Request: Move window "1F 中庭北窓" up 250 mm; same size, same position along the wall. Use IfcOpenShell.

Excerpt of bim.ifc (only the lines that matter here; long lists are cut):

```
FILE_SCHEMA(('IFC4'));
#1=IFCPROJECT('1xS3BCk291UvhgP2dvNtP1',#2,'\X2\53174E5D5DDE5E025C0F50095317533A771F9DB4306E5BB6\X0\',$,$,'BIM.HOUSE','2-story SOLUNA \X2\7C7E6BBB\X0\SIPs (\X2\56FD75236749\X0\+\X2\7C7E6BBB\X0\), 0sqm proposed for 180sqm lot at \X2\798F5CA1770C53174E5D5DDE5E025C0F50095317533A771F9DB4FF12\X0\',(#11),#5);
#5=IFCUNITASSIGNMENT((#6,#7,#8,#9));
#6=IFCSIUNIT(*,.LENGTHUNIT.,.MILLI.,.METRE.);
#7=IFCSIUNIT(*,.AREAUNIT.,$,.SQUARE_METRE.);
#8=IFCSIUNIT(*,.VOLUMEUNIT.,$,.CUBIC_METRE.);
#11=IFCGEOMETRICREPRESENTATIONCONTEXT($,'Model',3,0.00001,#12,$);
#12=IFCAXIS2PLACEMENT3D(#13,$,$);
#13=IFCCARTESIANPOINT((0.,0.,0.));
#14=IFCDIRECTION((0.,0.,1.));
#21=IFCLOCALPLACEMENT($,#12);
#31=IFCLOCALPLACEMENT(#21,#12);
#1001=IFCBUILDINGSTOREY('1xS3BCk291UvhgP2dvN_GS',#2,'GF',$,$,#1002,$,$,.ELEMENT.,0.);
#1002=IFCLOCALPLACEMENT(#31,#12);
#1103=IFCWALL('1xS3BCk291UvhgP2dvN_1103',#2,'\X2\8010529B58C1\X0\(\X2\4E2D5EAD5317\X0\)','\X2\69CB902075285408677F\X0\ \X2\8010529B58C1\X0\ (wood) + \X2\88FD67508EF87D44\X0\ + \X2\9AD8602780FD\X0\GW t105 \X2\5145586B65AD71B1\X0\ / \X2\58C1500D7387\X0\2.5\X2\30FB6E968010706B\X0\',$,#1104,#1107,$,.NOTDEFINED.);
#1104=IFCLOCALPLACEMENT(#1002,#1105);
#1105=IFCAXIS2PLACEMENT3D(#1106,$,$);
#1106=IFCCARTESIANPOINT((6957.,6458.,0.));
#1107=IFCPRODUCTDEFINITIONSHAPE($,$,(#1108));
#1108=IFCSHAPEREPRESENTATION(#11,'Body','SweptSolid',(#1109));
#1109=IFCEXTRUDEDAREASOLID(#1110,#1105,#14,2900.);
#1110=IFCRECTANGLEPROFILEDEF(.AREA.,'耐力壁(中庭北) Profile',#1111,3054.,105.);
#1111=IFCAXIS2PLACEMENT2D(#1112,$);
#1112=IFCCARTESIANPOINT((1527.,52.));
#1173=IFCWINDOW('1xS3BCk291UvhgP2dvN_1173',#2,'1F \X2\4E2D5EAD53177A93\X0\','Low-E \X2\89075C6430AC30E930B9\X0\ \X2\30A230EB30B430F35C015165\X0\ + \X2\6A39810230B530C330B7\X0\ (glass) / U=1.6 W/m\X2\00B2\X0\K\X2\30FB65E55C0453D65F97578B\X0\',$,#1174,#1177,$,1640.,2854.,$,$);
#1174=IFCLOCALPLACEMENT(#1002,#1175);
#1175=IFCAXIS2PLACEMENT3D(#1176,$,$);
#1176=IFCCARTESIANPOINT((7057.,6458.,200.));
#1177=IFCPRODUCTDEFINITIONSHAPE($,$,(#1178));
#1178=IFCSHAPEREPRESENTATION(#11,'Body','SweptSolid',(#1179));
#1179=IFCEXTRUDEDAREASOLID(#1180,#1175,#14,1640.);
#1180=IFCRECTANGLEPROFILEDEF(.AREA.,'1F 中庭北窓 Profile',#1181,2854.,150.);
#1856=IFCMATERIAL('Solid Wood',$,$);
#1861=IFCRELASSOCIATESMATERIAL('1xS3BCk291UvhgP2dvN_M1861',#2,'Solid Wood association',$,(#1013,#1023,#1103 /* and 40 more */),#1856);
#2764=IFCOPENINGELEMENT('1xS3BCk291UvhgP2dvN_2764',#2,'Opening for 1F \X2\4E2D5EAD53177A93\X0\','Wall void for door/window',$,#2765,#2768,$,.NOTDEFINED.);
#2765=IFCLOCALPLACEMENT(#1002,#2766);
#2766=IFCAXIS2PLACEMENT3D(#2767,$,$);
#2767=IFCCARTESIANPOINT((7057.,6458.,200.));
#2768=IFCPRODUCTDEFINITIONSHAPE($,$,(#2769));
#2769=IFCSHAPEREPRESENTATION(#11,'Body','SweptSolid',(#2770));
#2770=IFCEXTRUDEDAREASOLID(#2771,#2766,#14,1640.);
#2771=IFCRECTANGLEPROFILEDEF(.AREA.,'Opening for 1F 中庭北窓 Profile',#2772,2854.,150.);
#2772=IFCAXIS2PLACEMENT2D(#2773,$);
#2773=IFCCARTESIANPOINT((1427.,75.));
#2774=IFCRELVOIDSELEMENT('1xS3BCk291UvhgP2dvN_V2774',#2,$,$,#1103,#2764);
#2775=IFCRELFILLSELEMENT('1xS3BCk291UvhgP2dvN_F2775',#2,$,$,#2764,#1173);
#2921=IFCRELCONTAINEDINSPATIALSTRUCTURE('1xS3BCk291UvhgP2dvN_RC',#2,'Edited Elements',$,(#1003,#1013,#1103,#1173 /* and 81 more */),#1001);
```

```python
import numpy as np
import ifcopenshell
import ifcopenshell.api.geometry
import ifcopenshell.util.placement
import ifcopenshell.util.unit

model = ifcopenshell.open("bim.ifc")
unit_scale = ifcopenshell.util.unit.calculate_unit_scale(model)

window = model.by_guid("1xS3BCk291UvhgP2dvN_1173")
opening = window.FillsVoids[0].RelatingOpeningElement
dz = 0.25 / unit_scale

shift = np.array([0.0, 0.0, dz])
# The window is not placed relative to its opening, so move both.
for product in (opening, window):
    matrix = ifcopenshell.util.placement.get_local_placement(product.ObjectPlacement)
    matrix[:3, 3] += shift
    ifcopenshell.api.geometry.edit_object_placement(model, product=product, matrix=matrix, is_si=False)

print(f"moved by {dz * unit_scale:+.3f} m")

model.write("bim_v2.ifc")
```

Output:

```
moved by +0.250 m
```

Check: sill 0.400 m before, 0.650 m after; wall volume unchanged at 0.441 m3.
